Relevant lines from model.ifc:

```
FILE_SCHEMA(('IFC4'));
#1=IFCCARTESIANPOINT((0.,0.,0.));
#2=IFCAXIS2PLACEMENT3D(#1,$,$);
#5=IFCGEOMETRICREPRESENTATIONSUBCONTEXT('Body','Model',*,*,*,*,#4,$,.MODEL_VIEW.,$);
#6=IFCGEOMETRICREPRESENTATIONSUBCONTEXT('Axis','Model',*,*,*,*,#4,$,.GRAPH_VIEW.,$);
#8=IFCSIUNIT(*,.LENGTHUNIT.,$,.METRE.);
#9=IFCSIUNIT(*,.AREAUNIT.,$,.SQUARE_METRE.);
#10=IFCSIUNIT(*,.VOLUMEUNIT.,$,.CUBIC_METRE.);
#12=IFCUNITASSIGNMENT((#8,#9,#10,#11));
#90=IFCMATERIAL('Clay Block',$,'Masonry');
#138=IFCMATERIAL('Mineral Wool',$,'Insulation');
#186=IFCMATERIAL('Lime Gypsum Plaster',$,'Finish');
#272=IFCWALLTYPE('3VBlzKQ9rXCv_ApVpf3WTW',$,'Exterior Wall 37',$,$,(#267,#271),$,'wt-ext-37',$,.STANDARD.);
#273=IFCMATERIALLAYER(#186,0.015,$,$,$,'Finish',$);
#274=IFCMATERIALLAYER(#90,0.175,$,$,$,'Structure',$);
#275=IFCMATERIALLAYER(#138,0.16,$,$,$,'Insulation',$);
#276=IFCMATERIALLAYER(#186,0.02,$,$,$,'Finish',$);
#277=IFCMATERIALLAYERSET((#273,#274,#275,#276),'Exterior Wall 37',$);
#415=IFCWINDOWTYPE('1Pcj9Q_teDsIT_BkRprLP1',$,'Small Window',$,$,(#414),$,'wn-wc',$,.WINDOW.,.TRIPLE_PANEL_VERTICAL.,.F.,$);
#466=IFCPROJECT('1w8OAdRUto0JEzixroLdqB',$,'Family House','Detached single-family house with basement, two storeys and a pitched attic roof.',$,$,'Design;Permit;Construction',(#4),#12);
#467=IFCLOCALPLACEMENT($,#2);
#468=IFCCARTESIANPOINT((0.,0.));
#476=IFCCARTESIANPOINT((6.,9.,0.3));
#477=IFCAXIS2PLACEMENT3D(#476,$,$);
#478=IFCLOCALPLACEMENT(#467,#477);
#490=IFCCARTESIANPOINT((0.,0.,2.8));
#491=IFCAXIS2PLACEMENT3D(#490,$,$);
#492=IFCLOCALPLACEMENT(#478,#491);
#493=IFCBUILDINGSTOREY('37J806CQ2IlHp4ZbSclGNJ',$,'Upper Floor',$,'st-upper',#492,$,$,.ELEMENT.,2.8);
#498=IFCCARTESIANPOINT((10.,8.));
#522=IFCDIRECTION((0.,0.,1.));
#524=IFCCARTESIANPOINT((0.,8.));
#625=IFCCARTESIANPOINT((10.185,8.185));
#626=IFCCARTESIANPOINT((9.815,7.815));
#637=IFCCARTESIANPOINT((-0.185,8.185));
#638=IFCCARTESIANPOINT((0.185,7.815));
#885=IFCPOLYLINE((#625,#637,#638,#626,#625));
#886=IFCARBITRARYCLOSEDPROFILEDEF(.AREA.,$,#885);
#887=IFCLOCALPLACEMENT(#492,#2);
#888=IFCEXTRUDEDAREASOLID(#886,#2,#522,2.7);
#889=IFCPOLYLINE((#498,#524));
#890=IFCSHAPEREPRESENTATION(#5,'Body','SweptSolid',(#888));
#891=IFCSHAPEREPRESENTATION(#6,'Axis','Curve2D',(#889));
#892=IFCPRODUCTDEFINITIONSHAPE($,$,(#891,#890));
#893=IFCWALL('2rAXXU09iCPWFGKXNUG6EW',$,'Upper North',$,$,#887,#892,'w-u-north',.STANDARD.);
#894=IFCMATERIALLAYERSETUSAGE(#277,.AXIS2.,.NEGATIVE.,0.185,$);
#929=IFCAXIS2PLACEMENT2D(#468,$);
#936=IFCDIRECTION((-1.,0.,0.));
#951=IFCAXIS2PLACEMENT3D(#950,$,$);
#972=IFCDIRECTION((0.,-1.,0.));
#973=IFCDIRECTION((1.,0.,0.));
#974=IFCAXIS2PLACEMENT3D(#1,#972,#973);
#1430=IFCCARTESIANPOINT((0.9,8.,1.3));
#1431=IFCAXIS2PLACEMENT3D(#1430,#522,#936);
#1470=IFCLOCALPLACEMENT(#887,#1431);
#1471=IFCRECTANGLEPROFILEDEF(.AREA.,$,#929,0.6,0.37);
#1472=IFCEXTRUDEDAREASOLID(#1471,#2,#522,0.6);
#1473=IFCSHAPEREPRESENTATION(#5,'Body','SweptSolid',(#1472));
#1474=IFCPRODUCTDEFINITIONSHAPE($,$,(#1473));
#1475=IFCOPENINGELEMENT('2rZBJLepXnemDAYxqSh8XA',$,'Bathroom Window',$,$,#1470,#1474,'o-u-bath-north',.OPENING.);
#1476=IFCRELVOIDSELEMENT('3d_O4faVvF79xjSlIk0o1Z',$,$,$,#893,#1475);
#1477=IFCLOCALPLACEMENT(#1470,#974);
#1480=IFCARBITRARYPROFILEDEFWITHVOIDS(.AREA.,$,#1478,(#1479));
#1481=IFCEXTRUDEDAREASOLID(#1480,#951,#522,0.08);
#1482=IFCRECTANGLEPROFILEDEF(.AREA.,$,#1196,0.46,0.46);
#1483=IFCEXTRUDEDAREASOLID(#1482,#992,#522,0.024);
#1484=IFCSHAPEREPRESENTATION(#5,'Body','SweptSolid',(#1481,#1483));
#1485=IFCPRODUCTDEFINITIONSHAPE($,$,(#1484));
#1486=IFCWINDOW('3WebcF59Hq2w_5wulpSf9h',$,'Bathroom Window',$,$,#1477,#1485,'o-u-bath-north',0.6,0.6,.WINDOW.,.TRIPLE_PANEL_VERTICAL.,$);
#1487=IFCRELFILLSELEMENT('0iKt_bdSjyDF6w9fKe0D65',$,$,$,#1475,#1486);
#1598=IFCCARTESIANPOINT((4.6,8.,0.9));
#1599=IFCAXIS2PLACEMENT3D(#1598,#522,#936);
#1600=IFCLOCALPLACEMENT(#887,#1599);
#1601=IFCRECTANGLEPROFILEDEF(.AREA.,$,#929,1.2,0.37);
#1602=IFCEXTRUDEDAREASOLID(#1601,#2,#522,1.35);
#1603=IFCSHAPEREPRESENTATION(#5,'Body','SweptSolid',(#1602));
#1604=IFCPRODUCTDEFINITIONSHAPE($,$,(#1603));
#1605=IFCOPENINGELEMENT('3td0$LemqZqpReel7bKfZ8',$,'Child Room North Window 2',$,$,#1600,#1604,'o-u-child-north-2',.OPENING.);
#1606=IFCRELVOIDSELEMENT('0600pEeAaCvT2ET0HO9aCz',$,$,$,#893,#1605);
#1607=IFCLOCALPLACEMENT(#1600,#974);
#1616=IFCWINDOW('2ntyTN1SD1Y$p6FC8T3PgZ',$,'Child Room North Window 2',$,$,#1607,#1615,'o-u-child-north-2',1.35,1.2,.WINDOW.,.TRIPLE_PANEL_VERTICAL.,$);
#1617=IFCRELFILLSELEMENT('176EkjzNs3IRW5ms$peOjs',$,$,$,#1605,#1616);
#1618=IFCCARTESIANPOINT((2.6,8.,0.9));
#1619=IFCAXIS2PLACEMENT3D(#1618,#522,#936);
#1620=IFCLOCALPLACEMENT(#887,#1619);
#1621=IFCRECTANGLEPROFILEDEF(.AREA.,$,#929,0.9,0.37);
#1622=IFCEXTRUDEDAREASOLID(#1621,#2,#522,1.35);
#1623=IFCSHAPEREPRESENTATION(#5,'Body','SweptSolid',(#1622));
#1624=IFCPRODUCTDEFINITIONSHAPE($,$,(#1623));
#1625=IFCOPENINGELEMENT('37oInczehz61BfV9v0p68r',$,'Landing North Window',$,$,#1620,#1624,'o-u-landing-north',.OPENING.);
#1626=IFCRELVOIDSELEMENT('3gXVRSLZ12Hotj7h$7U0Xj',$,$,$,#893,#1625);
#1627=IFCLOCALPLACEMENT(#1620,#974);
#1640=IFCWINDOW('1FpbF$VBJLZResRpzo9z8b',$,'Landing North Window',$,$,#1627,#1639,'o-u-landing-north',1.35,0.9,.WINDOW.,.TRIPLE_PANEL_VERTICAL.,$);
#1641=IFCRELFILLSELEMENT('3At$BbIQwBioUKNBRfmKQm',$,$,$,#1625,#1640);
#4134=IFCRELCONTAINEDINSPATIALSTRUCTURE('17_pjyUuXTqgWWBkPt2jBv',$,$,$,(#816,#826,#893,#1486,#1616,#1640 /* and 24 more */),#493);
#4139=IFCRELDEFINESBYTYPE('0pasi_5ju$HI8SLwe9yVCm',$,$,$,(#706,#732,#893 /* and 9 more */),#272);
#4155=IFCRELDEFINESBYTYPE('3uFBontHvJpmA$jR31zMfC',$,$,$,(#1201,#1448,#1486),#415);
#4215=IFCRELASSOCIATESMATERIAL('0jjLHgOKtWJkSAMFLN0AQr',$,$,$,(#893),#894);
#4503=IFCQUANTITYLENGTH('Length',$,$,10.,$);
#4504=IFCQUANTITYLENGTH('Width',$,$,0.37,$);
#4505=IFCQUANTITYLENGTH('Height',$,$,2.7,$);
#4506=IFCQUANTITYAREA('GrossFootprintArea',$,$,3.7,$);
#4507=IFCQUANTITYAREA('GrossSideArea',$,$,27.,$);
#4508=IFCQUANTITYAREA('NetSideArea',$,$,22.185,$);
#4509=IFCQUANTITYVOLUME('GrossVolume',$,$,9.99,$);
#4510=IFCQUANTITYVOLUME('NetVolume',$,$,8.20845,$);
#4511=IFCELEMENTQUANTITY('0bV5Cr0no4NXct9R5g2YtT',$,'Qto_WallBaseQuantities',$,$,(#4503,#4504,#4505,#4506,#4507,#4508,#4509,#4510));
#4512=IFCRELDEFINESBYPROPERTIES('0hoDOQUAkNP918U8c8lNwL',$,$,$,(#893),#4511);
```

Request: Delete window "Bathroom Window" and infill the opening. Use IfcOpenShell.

```python
import ifcopenshell
import ifcopenshell.api.feature
import ifcopenshell.api.pset
import ifcopenshell.api.root
import ifcopenshell.geom
import ifcopenshell.util.element
import ifcopenshell.util.shape
import ifcopenshell.util.unit

model = ifcopenshell.open("model.ifc")
area_scale = ifcopenshell.util.unit.calculate_unit_scale(model, "AREAUNIT")
volume_scale = ifcopenshell.util.unit.calculate_unit_scale(model, "VOLUMEUNIT")
settings = ifcopenshell.geom.settings()


def volume(element):
    """Net volume in cubic metres, openings subtracted."""
    shape = ifcopenshell.geom.create_shape(settings, element)
    return ifcopenshell.util.shape.get_volume(shape.geometry)


window = model.by_id(1486)
opening = window.FillsVoids[0].RelatingOpeningElement
wall = opening.VoidsElements[0].RelatingBuildingElement
before = volume(wall)

ifcopenshell.api.root.remove_product(model, product=window)
ifcopenshell.api.feature.remove_feature(model, feature=opening)

after = volume(wall)
thickness = 0.37  # wall thickness in metres

# Update the wall's stored quantities.
qto = model.by_id(ifcopenshell.util.element.get_pset(wall, "Qto_WallBaseQuantities", should_inherit=False)["id"])
ifcopenshell.api.pset.edit_qto(model, qto=qto, properties={
    "NetSideArea": after / thickness / area_scale,
    "NetVolume": after / volume_scale,
})

print(f"wall volume {before:.3f} -> {after:.3f} m3")

model.write("model_v2.ifc")
```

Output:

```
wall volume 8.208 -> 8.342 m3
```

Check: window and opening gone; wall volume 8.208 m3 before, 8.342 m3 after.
